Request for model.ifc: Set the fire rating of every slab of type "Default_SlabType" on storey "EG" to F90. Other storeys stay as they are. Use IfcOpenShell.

First a look at what the model holds.

```python
import ifcopenshell
import ifcopenshell.util.element

model = ifcopenshell.open("model.ifc")
print(model.schema)
storey = next(s for s in model.by_type("IfcBuildingStorey") if s.Name == "EG")
slabs = [e for e in ifcopenshell.util.element.get_decomposition(storey) if e.is_a("IfcSlab")]
seen = {}
for e in slabs:
    element_type = ifcopenshell.util.element.get_type(e)
    key = (element_type.Name if element_type != e and element_type else None, ifcopenshell.util.element.get_pset(e, "Pset_SlabCommon", "FireRating"))
    seen[key] = seen.get(key, 0) + 1
for (name, value), count in sorted(seen.items(), key=str):
    print(count, "x", name, "|", value)
```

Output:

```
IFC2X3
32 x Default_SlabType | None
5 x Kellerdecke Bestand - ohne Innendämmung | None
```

```python
import ifcopenshell
import ifcopenshell.api.pset
import ifcopenshell.util.element

model = ifcopenshell.open("model.ifc")

storey = next(s for s in model.by_type("IfcBuildingStorey") if s.Name == "EG")
slabs = [e for e in ifcopenshell.util.element.get_decomposition(storey) if e.is_a("IfcSlab")]

count = 0
for e in slabs:
    element_type = ifcopenshell.util.element.get_type(e)
    if element_type in (None, e) or element_type.Name != "Default_SlabType":
        continue
    # add_pset returns the element's existing set when there is one.
    pset = ifcopenshell.api.pset.add_pset(model, product=e, name="Pset_SlabCommon")
    ifcopenshell.api.pset.edit_pset(model, pset=pset, properties={"FireRating": "F90"})
    count += 1

print(count, "slabs updated")

model.write("model_v2.ifc")
```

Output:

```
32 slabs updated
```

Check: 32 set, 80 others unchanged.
